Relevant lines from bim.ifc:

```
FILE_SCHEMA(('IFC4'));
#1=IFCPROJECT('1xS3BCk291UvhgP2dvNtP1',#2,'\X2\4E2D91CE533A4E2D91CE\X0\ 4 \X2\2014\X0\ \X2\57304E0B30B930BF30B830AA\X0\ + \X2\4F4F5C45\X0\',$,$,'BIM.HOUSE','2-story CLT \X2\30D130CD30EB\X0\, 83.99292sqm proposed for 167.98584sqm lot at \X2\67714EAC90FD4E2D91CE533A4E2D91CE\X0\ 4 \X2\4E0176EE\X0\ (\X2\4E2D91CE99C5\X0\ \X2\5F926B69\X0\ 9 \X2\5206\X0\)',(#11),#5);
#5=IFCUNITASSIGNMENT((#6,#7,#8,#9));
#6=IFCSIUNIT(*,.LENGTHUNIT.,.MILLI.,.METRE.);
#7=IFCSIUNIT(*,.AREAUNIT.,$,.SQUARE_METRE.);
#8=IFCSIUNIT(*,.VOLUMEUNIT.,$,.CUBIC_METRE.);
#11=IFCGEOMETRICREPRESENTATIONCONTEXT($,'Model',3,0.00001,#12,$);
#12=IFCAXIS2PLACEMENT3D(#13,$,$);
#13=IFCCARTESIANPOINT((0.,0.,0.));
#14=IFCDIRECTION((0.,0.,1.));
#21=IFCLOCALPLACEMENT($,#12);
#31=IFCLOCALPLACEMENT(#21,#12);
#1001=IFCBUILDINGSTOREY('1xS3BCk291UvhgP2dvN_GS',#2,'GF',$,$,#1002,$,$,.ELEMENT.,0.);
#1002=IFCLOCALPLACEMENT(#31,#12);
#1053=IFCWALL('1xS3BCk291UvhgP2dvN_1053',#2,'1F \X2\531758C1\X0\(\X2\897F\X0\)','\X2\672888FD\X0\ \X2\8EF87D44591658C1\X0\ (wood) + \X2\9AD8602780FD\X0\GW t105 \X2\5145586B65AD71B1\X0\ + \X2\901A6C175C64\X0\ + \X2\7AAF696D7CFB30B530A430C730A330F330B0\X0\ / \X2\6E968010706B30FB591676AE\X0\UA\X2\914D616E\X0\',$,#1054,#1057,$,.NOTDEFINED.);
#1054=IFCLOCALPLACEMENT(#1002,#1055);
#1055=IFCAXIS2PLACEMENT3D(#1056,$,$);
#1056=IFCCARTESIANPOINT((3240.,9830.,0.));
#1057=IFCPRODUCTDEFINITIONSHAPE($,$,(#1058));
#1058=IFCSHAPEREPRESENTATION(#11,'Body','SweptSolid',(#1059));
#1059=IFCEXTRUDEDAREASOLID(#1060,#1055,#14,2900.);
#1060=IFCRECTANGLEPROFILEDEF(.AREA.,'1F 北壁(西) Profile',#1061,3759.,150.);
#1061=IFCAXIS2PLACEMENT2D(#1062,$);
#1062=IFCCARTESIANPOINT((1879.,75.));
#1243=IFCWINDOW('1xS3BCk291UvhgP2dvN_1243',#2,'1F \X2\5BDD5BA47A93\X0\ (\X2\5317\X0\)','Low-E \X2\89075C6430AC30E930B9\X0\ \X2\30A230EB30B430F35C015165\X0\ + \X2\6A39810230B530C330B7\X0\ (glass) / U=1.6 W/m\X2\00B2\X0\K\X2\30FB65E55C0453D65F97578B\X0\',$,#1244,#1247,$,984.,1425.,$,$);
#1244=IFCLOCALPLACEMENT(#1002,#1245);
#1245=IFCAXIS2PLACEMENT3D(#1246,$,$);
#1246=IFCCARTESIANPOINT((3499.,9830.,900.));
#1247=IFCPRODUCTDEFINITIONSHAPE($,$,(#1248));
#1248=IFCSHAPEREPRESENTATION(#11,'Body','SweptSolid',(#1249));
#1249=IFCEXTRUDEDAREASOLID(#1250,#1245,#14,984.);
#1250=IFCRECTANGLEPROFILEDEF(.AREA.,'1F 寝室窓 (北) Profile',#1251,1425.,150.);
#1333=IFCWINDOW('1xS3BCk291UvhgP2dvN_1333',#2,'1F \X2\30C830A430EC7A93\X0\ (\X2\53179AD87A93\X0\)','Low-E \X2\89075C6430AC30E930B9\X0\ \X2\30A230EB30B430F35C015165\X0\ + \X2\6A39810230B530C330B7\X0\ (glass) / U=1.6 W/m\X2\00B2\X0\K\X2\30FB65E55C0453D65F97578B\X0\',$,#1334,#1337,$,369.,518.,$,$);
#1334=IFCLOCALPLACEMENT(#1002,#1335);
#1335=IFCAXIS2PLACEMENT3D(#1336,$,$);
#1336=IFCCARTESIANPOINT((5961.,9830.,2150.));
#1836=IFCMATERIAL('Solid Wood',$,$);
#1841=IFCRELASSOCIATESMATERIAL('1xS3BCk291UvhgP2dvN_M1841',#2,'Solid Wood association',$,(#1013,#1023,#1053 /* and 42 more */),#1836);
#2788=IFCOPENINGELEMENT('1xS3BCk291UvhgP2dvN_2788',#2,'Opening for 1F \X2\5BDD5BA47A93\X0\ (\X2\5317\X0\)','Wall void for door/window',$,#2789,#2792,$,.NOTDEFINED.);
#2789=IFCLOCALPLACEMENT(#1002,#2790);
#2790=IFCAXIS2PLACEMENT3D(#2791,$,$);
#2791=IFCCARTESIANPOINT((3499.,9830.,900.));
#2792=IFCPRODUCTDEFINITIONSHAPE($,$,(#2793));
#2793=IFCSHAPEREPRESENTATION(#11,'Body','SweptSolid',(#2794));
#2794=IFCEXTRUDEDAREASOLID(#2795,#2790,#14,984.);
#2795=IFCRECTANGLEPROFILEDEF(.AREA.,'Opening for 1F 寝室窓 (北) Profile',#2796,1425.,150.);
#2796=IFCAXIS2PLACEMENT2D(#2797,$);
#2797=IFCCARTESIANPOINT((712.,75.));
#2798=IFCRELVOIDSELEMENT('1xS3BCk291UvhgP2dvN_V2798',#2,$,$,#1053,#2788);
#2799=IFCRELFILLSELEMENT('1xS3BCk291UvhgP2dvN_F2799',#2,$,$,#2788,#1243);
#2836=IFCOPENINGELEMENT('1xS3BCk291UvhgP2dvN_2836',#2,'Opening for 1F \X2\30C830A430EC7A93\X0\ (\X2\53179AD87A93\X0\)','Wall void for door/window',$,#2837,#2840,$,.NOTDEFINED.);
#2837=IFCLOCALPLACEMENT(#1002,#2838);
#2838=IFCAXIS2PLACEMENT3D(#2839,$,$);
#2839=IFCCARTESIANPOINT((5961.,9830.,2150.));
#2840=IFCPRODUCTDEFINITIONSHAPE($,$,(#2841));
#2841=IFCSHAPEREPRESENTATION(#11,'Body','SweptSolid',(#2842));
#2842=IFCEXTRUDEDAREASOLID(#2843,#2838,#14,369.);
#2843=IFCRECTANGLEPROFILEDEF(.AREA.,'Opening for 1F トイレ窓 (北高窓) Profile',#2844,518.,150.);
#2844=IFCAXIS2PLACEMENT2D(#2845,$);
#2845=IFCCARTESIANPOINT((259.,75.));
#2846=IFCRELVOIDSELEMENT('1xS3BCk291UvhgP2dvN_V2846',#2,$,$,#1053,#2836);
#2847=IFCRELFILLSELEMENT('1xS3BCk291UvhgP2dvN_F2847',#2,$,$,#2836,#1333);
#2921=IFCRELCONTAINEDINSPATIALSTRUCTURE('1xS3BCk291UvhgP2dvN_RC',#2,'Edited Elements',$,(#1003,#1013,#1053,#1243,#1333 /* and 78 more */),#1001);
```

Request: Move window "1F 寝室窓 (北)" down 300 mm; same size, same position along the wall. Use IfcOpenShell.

```python
import numpy as np
import ifcopenshell
import ifcopenshell.api.geometry
import ifcopenshell.util.placement
import ifcopenshell.util.unit

model = ifcopenshell.open("bim.ifc")
unit_scale = ifcopenshell.util.unit.calculate_unit_scale(model)

window = model.by_guid("1xS3BCk291UvhgP2dvN_1243")
opening = window.FillsVoids[0].RelatingOpeningElement
dz = -0.3 / unit_scale

shift = np.array([0.0, 0.0, dz])
# The window is not placed relative to its opening, so move both.
for product in (opening, window):
    matrix = ifcopenshell.util.placement.get_local_placement(product.ObjectPlacement)
    matrix[:3, 3] += shift
    ifcopenshell.api.geometry.edit_object_placement(model, product=product, matrix=matrix, is_si=False)

print(f"moved by {dz * unit_scale:+.3f} m")

model.write("bim-out.ifc")
```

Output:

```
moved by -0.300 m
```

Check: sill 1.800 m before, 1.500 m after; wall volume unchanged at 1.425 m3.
